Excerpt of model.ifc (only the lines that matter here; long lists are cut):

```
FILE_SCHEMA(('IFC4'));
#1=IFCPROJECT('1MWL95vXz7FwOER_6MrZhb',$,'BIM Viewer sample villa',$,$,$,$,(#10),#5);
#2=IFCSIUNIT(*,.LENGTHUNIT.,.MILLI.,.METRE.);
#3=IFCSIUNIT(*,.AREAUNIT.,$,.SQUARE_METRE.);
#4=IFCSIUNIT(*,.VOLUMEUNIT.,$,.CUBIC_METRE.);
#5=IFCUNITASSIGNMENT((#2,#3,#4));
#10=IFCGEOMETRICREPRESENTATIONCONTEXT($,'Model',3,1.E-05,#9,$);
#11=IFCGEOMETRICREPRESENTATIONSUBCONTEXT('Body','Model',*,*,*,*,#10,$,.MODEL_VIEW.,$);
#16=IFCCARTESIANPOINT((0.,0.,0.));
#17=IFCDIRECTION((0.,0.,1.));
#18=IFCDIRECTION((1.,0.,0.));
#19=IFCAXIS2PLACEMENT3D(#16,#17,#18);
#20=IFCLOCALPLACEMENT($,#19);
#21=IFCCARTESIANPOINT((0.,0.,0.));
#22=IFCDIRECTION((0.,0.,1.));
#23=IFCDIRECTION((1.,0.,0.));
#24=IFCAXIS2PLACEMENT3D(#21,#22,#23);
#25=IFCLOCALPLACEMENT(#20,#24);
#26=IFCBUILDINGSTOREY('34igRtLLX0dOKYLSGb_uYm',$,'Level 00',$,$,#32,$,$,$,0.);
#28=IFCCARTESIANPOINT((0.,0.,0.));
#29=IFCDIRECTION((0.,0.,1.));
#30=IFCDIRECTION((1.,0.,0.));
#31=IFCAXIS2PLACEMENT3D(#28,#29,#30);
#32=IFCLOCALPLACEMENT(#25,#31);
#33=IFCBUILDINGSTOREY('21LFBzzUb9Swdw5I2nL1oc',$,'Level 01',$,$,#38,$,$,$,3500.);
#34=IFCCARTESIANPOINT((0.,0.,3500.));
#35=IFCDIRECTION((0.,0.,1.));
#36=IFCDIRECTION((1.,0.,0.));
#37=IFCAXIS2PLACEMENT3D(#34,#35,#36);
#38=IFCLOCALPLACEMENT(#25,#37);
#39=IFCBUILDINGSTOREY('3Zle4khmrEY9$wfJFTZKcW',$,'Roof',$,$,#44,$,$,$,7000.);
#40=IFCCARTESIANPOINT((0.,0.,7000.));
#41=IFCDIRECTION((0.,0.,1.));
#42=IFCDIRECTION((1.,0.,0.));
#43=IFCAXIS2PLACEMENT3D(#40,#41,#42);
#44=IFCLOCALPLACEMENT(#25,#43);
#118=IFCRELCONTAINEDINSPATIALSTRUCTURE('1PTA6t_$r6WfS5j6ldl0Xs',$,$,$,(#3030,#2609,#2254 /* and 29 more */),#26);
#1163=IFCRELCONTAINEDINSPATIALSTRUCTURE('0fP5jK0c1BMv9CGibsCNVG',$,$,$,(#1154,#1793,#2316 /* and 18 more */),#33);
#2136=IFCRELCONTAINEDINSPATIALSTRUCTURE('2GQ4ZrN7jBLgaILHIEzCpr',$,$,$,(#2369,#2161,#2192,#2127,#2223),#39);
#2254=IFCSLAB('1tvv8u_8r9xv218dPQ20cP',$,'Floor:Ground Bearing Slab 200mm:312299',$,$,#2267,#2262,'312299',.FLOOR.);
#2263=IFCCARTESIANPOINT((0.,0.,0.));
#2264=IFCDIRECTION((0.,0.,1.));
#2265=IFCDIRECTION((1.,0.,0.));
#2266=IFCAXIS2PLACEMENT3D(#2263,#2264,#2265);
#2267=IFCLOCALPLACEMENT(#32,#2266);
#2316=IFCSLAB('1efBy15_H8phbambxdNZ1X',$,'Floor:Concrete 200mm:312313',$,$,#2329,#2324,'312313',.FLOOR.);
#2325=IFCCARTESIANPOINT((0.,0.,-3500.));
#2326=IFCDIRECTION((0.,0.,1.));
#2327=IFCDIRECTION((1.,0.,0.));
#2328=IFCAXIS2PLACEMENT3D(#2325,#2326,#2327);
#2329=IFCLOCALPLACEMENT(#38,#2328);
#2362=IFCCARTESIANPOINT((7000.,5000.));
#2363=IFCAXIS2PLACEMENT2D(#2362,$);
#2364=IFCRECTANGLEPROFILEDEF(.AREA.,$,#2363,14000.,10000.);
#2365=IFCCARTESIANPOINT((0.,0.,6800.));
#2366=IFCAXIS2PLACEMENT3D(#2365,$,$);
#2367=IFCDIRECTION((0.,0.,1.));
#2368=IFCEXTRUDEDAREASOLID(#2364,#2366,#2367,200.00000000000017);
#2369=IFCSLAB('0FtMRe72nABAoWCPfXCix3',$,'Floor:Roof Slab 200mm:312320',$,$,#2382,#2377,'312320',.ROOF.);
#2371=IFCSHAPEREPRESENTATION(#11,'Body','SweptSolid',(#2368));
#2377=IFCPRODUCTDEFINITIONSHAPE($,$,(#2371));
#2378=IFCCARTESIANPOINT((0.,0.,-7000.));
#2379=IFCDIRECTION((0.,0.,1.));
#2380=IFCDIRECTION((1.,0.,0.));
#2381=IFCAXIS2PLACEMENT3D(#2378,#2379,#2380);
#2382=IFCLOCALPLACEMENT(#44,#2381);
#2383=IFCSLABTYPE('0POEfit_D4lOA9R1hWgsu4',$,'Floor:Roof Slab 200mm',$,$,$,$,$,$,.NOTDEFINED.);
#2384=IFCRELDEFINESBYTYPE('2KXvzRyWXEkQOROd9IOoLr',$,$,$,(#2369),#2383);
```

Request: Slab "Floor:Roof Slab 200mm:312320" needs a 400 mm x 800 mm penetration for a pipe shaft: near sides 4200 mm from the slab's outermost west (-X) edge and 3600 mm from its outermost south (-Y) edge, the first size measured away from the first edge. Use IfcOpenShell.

```python
import numpy as np
import ifcopenshell
import ifcopenshell.api.feature
import ifcopenshell.api.geometry
import ifcopenshell.api.root
import ifcopenshell.geom
import ifcopenshell.util.placement
import ifcopenshell.util.representation
import ifcopenshell.util.shape
import ifcopenshell.util.unit

model = ifcopenshell.open("model.ifc")
unit_scale = ifcopenshell.util.unit.calculate_unit_scale(model)
settings = ifcopenshell.geom.settings()


def volume(element):
    """Net volume in cubic metres, openings subtracted."""
    shape = ifcopenshell.geom.create_shape(settings, element)
    return ifcopenshell.util.shape.get_volume(shape.geometry)


slab = model.by_guid("0FtMRe72nABAoWCPfXCix3")
before = volume(slab)

# Extent in the slab's own axes, in metres. The edges named are its -X and -Y sides.
slab_shape = ifcopenshell.geom.create_shape(settings, slab)
vertices = ifcopenshell.util.shape.get_vertices(slab_shape.geometry)
x_min, y_min, bottom = vertices.min(axis=0)
top = vertices[:, 2].max()

opening = ifcopenshell.api.root.create_entity(model, ifc_class="IfcOpeningElement", name="Pipe shaft opening", predefined_type="OPENING")
context = ifcopenshell.util.representation.get_context(model, "Model", "Body", "MODEL_VIEW")
width, depth = 0.4, 0.8
outline = [(0.0, 0.0), (width, 0.0), (width, depth), (0.0, depth), (0.0, 0.0)]
# Overshoot both faces by 50 mm so the cut is clean.
shape = ifcopenshell.api.geometry.add_slab_representation(
    model, context=context, depth=top - bottom + 0.1, polyline=outline
)
ifcopenshell.api.geometry.assign_representation(model, product=opening, representation=shape)

matrix = ifcopenshell.util.placement.get_local_placement(slab.ObjectPlacement)
matrix[:, 3] = matrix @ np.append(np.array([x_min + 4.2, y_min + 3.6, bottom - 0.05]) / unit_scale, 1.0)
ifcopenshell.api.geometry.edit_object_placement(model, product=opening, matrix=matrix, is_si=False)
ifcopenshell.api.feature.add_feature(model, feature=opening, element=slab)

after = volume(slab)

print(f"slab volume {before:.3f} -> {after:.3f} m3")

model.write("model_edited.ifc")
```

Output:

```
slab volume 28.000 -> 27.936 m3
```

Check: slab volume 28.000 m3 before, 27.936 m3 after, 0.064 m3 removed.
